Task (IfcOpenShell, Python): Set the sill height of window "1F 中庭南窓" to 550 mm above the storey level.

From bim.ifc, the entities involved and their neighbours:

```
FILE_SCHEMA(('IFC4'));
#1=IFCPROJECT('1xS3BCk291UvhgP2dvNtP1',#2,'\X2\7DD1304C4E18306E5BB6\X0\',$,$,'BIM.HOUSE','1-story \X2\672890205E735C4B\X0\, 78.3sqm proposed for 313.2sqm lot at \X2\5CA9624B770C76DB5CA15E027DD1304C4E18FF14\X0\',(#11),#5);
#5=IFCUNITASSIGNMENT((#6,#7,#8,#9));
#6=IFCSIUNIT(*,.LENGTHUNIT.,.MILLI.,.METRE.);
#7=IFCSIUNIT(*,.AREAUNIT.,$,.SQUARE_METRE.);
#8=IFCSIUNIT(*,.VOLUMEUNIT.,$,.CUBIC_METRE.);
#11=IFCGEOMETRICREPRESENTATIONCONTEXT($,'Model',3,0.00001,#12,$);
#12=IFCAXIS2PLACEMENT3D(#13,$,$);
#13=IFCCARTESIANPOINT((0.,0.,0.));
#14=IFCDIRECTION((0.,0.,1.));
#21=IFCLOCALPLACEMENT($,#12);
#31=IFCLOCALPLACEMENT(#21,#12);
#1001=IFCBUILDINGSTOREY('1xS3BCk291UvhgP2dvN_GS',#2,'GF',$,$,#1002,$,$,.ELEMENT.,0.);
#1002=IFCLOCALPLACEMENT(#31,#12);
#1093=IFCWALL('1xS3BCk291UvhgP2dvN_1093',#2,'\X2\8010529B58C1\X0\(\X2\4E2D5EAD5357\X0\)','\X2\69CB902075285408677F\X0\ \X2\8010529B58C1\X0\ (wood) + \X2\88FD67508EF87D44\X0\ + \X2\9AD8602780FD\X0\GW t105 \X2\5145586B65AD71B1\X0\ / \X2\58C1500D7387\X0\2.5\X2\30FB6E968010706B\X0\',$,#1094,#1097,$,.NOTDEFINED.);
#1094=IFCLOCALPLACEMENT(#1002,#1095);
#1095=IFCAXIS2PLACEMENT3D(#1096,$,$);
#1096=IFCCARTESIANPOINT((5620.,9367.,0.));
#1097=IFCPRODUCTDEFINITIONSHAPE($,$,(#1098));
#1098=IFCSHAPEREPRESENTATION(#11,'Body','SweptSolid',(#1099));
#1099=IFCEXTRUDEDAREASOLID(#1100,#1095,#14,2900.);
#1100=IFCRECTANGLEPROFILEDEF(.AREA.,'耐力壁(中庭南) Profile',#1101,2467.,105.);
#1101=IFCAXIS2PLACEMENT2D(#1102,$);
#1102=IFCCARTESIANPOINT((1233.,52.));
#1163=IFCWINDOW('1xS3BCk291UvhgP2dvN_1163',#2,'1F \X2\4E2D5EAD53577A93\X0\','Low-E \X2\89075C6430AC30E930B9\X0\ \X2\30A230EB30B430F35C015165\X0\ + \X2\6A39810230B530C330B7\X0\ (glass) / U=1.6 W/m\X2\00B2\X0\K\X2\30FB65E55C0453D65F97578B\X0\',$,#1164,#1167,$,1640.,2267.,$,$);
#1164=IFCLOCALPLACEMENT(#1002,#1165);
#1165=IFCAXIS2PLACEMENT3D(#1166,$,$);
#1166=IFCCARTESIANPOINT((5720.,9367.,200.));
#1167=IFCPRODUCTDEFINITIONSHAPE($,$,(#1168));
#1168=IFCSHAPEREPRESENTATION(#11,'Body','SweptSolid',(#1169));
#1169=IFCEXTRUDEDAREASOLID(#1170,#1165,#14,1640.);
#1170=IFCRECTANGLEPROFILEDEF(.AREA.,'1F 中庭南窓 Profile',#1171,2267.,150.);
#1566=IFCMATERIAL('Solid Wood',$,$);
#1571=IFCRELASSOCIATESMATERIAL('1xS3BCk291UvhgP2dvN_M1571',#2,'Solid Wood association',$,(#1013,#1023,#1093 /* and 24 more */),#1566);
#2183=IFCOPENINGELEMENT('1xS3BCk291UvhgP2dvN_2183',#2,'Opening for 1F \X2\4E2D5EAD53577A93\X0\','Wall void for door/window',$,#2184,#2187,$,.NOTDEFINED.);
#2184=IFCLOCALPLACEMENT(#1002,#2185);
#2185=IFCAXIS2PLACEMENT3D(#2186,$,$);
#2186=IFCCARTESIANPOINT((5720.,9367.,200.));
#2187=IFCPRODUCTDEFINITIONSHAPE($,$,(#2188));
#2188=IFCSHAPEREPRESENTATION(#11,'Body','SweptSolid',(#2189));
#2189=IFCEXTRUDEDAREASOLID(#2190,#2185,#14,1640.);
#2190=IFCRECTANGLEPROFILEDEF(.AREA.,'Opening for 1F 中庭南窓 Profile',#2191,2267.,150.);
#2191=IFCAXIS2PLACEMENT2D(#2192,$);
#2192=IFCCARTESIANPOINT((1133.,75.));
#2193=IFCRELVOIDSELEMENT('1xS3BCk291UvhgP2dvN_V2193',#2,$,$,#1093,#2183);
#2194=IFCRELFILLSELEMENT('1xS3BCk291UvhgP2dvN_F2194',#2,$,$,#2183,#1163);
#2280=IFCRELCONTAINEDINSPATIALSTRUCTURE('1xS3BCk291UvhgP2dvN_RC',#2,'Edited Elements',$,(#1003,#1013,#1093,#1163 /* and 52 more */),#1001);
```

```python
import numpy as np
import ifcopenshell
import ifcopenshell.api.geometry
import ifcopenshell.geom
import ifcopenshell.util.element
import ifcopenshell.util.placement
import ifcopenshell.util.shape
import ifcopenshell.util.unit

model = ifcopenshell.open("bim.ifc")
unit_scale = ifcopenshell.util.unit.calculate_unit_scale(model)

window = model.by_guid("1xS3BCk291UvhgP2dvN_1163")
opening = window.FillsVoids[0].RelatingOpeningElement
storey = ifcopenshell.util.element.get_container(window, ifc_class="IfcBuildingStorey")
level = ifcopenshell.util.placement.get_local_placement(storey.ObjectPlacement)[2, 3]

# The opening's origin need not be at the sill, so measure its lowest point.
shape = ifcopenshell.geom.create_shape(ifcopenshell.geom.settings(), opening)
bottom = ifcopenshell.util.shape.get_shape_bottom_elevation(shape, shape.geometry) / unit_scale
dz = level + 0.55 / unit_scale - bottom

shift = np.array([0.0, 0.0, dz])
# The window is not placed relative to its opening, so move both.
for product in (opening, window):
    matrix = ifcopenshell.util.placement.get_local_placement(product.ObjectPlacement)
    matrix[:3, 3] += shift
    ifcopenshell.api.geometry.edit_object_placement(model, product=product, matrix=matrix, is_si=False)

print(f"moved by {dz * unit_scale:+.3f} m")

model.write("bim_edited.ifc")
```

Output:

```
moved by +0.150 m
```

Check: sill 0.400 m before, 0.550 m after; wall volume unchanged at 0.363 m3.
